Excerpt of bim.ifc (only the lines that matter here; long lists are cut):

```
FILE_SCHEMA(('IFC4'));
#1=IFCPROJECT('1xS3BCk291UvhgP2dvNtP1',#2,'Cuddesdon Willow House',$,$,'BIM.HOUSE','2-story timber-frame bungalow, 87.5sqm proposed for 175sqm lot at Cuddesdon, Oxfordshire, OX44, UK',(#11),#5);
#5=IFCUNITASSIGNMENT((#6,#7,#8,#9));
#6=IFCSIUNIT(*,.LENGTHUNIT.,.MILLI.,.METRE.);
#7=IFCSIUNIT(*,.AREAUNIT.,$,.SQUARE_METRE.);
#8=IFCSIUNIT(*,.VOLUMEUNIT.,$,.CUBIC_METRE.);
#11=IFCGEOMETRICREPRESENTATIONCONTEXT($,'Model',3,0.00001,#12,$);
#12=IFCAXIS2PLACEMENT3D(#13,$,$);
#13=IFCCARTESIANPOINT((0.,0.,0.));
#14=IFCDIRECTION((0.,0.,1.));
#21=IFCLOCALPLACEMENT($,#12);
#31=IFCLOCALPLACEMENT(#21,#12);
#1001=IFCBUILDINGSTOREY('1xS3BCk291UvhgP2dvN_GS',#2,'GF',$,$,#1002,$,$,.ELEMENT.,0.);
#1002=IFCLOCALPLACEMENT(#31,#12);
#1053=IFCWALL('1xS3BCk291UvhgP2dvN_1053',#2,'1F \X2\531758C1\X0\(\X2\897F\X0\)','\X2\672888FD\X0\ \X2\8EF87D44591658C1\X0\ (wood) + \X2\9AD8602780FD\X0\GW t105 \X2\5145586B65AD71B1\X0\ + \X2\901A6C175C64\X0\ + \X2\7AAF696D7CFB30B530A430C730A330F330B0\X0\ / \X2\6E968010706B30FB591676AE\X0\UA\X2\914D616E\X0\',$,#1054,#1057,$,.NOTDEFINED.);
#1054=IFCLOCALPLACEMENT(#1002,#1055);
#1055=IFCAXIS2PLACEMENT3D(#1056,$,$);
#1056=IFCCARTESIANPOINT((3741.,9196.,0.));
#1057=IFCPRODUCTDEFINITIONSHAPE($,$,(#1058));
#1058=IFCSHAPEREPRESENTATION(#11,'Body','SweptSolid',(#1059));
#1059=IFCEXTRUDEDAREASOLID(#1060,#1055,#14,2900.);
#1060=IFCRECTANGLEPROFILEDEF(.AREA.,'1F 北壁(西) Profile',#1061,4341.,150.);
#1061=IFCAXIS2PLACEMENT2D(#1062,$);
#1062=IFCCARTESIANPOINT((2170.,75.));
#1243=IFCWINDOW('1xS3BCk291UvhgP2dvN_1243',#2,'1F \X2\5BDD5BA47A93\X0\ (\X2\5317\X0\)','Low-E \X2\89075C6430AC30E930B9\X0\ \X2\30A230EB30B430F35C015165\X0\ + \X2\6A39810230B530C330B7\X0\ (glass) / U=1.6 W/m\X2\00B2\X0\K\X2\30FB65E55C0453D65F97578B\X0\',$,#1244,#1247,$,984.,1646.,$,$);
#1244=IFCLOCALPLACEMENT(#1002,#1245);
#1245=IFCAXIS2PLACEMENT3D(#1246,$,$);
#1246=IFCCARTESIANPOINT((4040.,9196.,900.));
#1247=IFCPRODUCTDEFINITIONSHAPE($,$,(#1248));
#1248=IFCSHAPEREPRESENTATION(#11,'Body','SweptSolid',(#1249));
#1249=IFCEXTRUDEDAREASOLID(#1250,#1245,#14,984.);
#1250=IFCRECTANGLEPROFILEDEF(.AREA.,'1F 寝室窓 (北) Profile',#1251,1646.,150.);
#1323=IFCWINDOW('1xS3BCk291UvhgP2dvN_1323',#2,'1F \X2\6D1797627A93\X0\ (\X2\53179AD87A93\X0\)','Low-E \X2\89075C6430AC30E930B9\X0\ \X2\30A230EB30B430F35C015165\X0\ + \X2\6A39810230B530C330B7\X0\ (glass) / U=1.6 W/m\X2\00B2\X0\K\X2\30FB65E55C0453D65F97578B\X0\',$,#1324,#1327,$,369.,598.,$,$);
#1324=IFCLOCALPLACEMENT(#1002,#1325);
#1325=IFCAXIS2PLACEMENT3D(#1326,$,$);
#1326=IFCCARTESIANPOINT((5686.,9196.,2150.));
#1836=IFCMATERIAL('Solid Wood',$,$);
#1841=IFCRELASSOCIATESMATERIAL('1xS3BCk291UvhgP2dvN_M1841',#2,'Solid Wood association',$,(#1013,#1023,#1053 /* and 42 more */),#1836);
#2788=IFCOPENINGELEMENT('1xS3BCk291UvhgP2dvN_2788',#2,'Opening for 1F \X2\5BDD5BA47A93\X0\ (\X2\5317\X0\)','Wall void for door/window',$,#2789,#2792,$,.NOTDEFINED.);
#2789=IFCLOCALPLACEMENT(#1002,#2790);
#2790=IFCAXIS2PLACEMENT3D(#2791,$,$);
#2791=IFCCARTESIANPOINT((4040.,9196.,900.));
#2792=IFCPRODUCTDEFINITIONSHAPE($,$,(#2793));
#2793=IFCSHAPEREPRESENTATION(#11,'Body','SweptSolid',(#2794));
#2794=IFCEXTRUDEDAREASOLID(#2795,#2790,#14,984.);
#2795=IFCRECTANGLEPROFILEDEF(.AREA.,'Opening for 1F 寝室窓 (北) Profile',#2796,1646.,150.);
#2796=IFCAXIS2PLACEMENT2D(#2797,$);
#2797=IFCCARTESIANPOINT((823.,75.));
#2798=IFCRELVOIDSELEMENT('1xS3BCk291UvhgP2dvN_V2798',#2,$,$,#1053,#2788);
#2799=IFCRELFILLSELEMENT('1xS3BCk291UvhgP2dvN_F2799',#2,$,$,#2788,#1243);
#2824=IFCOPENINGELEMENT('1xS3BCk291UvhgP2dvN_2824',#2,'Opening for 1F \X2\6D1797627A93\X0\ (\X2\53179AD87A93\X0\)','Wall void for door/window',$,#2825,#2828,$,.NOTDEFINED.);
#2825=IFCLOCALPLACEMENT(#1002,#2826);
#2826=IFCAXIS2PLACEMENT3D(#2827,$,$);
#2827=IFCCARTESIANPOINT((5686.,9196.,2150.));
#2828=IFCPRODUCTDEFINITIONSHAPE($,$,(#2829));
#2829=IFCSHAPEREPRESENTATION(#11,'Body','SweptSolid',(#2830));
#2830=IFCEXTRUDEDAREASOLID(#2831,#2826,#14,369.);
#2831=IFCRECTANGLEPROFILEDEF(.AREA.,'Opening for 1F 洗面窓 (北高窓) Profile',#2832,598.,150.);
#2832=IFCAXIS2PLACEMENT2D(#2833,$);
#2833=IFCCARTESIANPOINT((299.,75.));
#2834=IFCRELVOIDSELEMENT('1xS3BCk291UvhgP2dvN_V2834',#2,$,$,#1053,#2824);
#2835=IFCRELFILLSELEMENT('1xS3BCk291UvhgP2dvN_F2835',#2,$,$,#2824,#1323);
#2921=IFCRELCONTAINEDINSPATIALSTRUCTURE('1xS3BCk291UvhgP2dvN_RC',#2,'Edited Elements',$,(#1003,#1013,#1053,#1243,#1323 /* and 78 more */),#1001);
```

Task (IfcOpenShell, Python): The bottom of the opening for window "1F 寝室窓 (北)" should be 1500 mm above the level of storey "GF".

```python
import numpy as np
import ifcopenshell
import ifcopenshell.api.geometry
import ifcopenshell.geom
import ifcopenshell.util.element
import ifcopenshell.util.placement
import ifcopenshell.util.shape
import ifcopenshell.util.unit

model = ifcopenshell.open("bim.ifc")
unit_scale = ifcopenshell.util.unit.calculate_unit_scale(model)

window = model.by_id(1243)
opening = window.FillsVoids[0].RelatingOpeningElement
storey = ifcopenshell.util.element.get_container(window, ifc_class="IfcBuildingStorey")
level = ifcopenshell.util.placement.get_local_placement(storey.ObjectPlacement)[2, 3]

# The opening's origin need not be at the sill, so measure its lowest point.
shape = ifcopenshell.geom.create_shape(ifcopenshell.geom.settings(), opening)
bottom = ifcopenshell.util.shape.get_shape_bottom_elevation(shape, shape.geometry) / unit_scale
dz = level + 1500.0 - bottom

shift = np.array([0.0, 0.0, dz])
# The window is not placed relative to its opening, so move both.
for product in (opening, window):
    matrix = ifcopenshell.util.placement.get_local_placement(product.ObjectPlacement)
    matrix[:3, 3] += shift
    ifcopenshell.api.geometry.edit_object_placement(model, product=product, matrix=matrix, is_si=False)

print(f"moved by {dz * unit_scale:+.3f} m")

model.write("bim_v2.ifc")
```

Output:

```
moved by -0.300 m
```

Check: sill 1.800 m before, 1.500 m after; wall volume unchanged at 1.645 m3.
